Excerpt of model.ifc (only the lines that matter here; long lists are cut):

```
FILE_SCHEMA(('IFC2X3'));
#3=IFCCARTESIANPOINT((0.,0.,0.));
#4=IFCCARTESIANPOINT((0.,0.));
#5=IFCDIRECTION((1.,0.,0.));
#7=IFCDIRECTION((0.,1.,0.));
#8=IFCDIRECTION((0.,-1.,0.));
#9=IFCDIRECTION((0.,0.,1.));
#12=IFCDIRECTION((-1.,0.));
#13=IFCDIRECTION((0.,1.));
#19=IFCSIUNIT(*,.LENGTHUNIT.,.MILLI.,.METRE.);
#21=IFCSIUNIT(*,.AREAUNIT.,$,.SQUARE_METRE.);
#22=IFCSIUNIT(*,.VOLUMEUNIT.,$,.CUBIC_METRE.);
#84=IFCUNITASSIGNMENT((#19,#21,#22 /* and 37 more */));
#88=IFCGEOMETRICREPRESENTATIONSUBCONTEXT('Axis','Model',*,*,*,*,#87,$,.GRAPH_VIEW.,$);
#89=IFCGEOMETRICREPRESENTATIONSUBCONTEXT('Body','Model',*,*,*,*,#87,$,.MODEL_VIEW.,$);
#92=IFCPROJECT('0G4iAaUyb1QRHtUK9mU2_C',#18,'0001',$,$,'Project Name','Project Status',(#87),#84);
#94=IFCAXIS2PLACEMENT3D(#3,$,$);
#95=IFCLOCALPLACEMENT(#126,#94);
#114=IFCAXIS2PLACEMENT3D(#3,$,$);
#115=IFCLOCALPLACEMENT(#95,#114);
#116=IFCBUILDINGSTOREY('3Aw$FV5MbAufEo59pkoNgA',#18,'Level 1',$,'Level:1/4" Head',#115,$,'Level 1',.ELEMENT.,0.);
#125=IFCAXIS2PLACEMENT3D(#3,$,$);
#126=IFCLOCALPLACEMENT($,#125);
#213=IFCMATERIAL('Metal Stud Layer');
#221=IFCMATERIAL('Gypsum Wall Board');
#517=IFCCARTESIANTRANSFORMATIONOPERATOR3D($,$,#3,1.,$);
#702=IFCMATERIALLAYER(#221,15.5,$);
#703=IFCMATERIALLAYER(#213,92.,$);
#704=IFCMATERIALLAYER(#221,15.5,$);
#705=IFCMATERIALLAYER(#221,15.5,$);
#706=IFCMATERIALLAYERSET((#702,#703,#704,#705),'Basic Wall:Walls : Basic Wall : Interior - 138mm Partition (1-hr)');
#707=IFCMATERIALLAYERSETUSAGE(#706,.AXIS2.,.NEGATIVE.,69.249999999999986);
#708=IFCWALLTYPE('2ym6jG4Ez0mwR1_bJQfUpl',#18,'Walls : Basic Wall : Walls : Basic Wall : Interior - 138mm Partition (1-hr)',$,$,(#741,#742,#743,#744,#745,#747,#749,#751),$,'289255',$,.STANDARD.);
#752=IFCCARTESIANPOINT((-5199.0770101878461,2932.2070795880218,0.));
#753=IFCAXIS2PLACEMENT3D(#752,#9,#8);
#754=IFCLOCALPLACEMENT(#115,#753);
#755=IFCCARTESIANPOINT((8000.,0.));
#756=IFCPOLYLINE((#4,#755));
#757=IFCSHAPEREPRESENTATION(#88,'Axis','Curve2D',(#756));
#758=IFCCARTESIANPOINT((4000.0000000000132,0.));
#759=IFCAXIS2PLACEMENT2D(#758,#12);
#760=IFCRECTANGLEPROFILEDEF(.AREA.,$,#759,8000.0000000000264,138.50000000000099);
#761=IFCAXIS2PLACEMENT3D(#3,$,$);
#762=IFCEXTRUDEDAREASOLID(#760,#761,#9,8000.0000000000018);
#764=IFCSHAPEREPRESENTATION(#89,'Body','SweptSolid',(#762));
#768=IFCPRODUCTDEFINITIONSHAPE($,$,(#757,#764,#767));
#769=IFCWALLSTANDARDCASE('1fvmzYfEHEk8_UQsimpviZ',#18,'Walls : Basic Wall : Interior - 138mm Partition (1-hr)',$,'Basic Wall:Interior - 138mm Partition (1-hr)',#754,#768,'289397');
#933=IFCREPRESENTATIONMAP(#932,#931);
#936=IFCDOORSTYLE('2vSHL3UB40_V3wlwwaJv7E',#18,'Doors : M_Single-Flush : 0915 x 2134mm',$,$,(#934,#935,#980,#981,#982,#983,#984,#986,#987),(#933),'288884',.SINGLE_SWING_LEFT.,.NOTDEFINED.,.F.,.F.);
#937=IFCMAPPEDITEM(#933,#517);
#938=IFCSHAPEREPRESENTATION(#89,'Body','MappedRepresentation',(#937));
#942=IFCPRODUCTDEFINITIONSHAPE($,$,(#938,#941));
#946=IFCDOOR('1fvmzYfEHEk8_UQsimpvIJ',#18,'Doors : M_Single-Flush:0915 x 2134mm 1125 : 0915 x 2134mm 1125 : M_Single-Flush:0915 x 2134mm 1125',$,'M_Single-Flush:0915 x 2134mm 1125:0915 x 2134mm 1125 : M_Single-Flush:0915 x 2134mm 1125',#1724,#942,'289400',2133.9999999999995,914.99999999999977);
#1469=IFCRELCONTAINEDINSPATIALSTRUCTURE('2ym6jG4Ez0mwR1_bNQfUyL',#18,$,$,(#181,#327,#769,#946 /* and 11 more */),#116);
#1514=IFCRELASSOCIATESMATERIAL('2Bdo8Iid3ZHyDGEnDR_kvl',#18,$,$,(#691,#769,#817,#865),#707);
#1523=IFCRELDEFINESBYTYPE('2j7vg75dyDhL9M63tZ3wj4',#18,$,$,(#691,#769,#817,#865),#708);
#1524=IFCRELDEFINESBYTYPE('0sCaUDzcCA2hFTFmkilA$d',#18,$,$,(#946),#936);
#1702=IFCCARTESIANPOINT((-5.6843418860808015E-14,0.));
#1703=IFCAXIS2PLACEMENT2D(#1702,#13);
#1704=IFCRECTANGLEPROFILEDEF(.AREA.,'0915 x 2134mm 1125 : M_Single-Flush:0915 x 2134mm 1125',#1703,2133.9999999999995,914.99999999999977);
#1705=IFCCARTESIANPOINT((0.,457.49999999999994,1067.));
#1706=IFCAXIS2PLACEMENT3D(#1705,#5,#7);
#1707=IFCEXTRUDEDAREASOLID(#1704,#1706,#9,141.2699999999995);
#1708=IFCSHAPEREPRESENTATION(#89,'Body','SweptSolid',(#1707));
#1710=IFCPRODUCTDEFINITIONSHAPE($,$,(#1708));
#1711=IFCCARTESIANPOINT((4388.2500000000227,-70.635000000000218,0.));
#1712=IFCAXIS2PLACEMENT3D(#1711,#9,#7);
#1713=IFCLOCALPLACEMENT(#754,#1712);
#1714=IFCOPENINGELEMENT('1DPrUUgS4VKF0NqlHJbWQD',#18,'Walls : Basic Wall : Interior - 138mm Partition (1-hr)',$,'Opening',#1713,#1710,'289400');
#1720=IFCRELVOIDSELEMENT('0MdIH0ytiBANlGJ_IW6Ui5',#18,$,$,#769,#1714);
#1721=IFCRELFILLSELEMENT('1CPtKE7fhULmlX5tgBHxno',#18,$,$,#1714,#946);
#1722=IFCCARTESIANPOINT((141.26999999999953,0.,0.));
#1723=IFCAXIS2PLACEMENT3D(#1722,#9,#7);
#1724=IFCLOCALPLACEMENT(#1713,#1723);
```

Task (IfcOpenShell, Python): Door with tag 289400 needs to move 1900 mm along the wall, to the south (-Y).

```python
import ifcopenshell
import ifcopenshell.api.geometry
import ifcopenshell.util.placement
import ifcopenshell.util.unit

model = ifcopenshell.open("model.ifc")
unit_scale = ifcopenshell.util.unit.calculate_unit_scale(model)

door = model.by_id(946)
opening = door.FillsVoids[0].RelatingOpeningElement
wall = opening.VoidsElements[0].RelatingBuildingElement

wall_matrix = ifcopenshell.util.placement.get_local_placement(wall.ObjectPlacement)
shift = wall_matrix[:3, 0] * 1.9 / unit_scale
before = ifcopenshell.util.placement.get_local_placement(door.ObjectPlacement)[:3, 3].copy()

# The door is placed relative to its opening, so it follows when the opening moves.
matrix = ifcopenshell.util.placement.get_local_placement(opening.ObjectPlacement)
matrix[:3, 3] += shift
ifcopenshell.api.geometry.edit_object_placement(
    model, product=opening, matrix=matrix, is_si=False, should_transform_children=True
)

after = ifcopenshell.util.placement.get_local_placement(door.ObjectPlacement)[:3, 3]
print("door moved by", (after - before).round(3) + 0.0)

model.write("model_v2.ifc")
```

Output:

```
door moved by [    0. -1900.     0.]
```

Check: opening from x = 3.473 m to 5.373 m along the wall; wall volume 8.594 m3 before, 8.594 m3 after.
